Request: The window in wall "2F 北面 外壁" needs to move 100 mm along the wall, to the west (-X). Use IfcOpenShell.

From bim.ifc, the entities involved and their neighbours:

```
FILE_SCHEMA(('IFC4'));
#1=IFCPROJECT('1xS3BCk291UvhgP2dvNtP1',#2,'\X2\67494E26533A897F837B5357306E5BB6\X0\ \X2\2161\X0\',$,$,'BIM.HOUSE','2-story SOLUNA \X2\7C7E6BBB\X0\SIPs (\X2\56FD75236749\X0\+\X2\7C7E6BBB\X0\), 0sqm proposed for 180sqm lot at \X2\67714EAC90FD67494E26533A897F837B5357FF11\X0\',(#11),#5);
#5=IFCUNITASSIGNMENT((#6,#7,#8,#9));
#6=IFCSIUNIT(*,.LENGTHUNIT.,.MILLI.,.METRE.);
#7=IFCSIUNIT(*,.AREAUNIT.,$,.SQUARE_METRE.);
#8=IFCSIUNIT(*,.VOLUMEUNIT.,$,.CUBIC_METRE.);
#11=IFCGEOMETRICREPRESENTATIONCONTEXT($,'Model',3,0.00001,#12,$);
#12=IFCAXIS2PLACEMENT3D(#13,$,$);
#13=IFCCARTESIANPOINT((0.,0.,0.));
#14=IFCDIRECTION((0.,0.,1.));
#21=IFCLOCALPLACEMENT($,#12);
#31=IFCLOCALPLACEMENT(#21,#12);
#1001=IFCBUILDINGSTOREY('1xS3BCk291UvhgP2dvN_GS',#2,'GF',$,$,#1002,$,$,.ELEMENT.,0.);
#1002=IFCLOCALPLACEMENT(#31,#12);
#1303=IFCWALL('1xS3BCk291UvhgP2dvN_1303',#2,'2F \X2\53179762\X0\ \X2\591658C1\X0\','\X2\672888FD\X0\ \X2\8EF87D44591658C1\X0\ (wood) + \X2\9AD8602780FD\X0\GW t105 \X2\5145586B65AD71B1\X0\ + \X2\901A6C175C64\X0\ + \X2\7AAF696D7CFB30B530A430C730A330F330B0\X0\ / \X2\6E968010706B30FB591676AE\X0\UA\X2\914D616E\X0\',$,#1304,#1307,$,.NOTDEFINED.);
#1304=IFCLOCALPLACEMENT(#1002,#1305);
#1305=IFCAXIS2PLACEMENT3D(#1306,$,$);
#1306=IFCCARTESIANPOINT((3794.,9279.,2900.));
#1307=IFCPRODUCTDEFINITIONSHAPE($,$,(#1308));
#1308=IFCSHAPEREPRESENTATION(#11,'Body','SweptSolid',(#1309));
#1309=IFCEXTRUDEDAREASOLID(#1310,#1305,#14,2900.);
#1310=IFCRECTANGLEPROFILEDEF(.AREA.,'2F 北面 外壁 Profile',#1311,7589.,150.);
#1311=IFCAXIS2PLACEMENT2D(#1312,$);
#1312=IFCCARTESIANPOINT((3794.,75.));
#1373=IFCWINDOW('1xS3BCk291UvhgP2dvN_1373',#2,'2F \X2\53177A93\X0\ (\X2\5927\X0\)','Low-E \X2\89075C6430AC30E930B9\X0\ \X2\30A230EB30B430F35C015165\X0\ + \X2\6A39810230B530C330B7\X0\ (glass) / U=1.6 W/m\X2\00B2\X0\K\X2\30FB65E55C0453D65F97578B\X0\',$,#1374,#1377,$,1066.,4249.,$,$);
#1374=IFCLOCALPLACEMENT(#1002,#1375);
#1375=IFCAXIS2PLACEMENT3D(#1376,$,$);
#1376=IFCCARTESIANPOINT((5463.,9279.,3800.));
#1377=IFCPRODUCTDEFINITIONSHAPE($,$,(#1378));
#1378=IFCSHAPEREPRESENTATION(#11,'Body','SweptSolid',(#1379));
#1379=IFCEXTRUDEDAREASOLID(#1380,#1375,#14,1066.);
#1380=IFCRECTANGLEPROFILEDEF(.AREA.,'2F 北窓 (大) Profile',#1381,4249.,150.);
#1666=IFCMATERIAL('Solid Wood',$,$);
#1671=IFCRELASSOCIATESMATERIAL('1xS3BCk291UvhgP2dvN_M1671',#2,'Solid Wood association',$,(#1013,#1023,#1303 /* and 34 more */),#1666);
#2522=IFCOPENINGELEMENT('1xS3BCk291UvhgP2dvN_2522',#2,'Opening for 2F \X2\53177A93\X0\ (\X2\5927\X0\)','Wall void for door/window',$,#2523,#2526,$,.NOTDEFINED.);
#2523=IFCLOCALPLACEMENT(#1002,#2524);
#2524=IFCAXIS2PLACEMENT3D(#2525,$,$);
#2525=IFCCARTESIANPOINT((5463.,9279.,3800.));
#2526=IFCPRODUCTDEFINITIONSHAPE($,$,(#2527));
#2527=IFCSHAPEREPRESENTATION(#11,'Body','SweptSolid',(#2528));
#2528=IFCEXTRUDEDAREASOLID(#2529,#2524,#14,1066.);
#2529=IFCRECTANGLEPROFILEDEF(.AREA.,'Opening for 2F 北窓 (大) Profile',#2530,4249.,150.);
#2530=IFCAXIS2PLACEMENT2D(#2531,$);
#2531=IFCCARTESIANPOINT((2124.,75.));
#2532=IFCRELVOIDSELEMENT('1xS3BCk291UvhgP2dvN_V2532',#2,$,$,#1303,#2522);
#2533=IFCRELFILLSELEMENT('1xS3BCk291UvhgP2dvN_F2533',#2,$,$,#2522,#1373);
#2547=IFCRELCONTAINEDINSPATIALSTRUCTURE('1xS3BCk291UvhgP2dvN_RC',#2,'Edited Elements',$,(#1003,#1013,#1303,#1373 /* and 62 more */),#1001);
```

```python
import ifcopenshell
import ifcopenshell.api.geometry
import ifcopenshell.util.placement
import ifcopenshell.util.unit

model = ifcopenshell.open("bim.ifc")
unit_scale = ifcopenshell.util.unit.calculate_unit_scale(model)

window = model.by_id(1373)
opening = window.FillsVoids[0].RelatingOpeningElement
wall = opening.VoidsElements[0].RelatingBuildingElement

wall_matrix = ifcopenshell.util.placement.get_local_placement(wall.ObjectPlacement)
shift = wall_matrix[:3, 0] * -0.1 / unit_scale
before = ifcopenshell.util.placement.get_local_placement(window.ObjectPlacement)[:3, 3].copy()

# The window is not placed relative to its opening, so move both.
for product in (opening, window):
    matrix = ifcopenshell.util.placement.get_local_placement(product.ObjectPlacement)
    matrix[:3, 3] += shift
    ifcopenshell.api.geometry.edit_object_placement(model, product=product, matrix=matrix, is_si=False)

after = ifcopenshell.util.placement.get_local_placement(window.ObjectPlacement)[:3, 3]
print("window moved by", (after - before).round(3) + 0.0)

model.write("bim-out.ifc")
```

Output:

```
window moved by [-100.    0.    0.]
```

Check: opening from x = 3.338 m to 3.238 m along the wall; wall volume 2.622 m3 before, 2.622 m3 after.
